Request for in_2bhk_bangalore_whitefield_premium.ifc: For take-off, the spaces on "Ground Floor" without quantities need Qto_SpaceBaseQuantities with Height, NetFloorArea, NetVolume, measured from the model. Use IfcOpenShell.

First a look at what the model holds.

```python
import ifcopenshell
import ifcopenshell.util.element
import ifcopenshell.util.unit

model = ifcopenshell.open("in_2bhk_bangalore_whitefield_premium.ifc")
print(model.schema)
for unit_type in ("LENGTHUNIT", "AREAUNIT", "VOLUMEUNIT"):
    print(unit_type, ifcopenshell.util.unit.calculate_unit_scale(model, unit_type))
storey = next(s for s in model.by_type("IfcBuildingStorey") if s.Name == "Ground Floor")
spaces = [e for e in ifcopenshell.util.element.get_decomposition(storey) if e.is_a("IfcSpace")]
for e in sorted(spaces, key=lambda e: e.id()):
    print(e.id(), e.is_a(), e.Name, list(ifcopenshell.util.element.get_psets(e, qtos_only=True)), sep=" | ")
```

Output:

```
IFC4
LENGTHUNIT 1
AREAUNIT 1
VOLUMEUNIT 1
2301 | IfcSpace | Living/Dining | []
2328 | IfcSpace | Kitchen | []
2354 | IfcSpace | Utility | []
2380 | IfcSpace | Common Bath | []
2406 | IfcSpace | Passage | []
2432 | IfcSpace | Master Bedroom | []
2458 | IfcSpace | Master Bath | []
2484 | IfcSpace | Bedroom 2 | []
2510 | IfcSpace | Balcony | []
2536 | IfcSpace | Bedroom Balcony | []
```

```python
import ifcopenshell
import ifcopenshell.api.pset
import ifcopenshell.geom
import ifcopenshell.util.element
import ifcopenshell.util.shape
import ifcopenshell.util.unit

model = ifcopenshell.open("in_2bhk_bangalore_whitefield_premium.ifc")
unit_scale = ifcopenshell.util.unit.calculate_unit_scale(model)
area_scale = ifcopenshell.util.unit.calculate_unit_scale(model, "AREAUNIT")
volume_scale = ifcopenshell.util.unit.calculate_unit_scale(model, "VOLUMEUNIT")
settings = ifcopenshell.geom.settings()

storey = next(s for s in model.by_type("IfcBuildingStorey") if s.Name == "Ground Floor")
spaces = [e for e in ifcopenshell.util.element.get_decomposition(storey) if e.is_a("IfcSpace")]

for e in sorted(spaces, key=lambda e: e.id()):
    if ifcopenshell.util.element.get_psets(e, qtos_only=True, should_inherit=False):
        continue
    # Geometry comes back in metres, in the element's own axes.
    shape = ifcopenshell.geom.create_shape(settings, e)
    values = {
        "Height": ifcopenshell.util.shape.get_z(shape.geometry) / unit_scale,
        "NetFloorArea": ifcopenshell.util.shape.get_footprint_area(shape.geometry) / area_scale,
        "NetVolume": ifcopenshell.util.shape.get_volume(shape.geometry) / volume_scale,
    }
    qto = ifcopenshell.api.pset.add_qto(model, product=e, name="Qto_SpaceBaseQuantities")
    ifcopenshell.api.pset.edit_qto(model, qto=qto, properties=values)
    print(e.id(), {k: round(v, 3) for k, v in values.items()})

model.write("in_2bhk_bangalore_whitefield_premium_edited.ifc")
```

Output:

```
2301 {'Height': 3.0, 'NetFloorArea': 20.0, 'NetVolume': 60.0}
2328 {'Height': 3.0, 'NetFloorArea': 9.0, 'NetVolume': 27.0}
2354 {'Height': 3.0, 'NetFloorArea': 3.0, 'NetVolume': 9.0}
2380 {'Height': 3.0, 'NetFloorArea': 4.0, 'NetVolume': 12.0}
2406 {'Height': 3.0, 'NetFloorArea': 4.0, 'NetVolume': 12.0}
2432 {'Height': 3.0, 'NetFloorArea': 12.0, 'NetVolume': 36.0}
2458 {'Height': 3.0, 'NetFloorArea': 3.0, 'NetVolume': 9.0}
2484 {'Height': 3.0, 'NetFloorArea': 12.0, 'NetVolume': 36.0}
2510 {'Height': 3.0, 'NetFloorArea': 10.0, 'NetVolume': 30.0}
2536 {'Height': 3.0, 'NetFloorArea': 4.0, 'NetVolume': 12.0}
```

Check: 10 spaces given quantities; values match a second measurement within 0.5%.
